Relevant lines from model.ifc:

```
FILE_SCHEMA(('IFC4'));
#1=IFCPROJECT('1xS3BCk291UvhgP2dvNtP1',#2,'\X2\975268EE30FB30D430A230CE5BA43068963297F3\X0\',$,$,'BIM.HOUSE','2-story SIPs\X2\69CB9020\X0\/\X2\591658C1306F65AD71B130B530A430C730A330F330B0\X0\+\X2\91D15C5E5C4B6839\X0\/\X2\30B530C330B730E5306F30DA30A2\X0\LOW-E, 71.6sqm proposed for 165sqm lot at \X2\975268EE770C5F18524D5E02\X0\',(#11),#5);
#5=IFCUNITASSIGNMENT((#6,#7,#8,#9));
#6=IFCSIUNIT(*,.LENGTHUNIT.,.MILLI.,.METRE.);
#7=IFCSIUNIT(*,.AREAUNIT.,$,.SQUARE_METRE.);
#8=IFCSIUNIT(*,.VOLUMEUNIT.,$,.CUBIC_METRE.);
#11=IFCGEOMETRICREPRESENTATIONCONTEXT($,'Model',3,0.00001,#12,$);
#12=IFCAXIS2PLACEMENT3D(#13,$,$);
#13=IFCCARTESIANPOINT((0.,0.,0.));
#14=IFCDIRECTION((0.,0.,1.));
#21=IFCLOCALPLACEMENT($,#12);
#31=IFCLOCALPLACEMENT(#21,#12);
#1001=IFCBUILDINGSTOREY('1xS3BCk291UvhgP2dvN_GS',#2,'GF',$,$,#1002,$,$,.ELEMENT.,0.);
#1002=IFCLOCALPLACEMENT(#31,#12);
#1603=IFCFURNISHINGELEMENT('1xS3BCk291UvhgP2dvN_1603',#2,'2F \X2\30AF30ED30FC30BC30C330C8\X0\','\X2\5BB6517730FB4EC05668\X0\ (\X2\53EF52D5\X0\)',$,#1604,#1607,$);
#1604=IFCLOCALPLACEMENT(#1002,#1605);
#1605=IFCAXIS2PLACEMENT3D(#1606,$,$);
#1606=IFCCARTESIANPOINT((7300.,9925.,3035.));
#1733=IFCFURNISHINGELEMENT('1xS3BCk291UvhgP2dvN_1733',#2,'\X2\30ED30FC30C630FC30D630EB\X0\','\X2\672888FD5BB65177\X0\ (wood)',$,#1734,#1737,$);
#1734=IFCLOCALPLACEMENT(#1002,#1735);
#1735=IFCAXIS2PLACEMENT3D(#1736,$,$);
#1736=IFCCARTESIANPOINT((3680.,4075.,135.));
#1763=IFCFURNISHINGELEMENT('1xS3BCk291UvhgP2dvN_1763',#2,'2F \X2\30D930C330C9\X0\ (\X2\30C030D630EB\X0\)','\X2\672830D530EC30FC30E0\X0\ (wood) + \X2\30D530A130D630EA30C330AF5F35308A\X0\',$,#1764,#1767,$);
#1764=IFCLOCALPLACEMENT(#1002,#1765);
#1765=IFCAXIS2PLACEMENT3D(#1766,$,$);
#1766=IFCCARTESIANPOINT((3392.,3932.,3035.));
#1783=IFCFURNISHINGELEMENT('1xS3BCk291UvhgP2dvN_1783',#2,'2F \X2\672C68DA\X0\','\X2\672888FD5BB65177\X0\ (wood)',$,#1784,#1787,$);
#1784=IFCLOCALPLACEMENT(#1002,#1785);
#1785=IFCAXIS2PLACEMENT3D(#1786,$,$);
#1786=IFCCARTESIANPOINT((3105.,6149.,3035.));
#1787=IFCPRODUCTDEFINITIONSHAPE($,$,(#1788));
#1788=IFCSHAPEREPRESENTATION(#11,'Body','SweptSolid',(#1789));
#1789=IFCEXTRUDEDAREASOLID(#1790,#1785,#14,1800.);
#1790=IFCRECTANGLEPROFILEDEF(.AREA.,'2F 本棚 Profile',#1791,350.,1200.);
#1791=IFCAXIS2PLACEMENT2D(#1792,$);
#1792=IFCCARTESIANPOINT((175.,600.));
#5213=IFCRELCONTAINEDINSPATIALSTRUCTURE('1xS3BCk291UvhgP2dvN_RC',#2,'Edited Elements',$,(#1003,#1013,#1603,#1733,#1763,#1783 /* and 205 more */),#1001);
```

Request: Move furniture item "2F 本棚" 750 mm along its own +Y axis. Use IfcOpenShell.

```python
import ifcopenshell
import ifcopenshell.api.geometry
import ifcopenshell.util.placement
import ifcopenshell.util.unit

model = ifcopenshell.open("model.ifc")
unit_scale = ifcopenshell.util.unit.calculate_unit_scale(model)

item = model.by_guid("1xS3BCk291UvhgP2dvN_1783")
matrix = ifcopenshell.util.placement.get_local_placement(item.ObjectPlacement)
matrix[:3, 3] += matrix[:3, 1] * 0.75 / unit_scale
ifcopenshell.api.geometry.edit_object_placement(model, product=item, matrix=matrix, is_si=False)

print(ifcopenshell.util.placement.get_local_placement(item.ObjectPlacement).round(3) + 0.0)

model.write("model_rev.ifc")
```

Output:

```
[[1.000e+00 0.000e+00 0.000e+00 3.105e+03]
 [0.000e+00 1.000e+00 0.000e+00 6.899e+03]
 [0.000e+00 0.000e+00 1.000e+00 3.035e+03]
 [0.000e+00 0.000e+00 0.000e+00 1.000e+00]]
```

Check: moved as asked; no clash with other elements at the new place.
